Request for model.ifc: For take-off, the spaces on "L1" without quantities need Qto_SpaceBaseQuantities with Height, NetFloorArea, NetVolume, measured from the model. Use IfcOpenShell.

First a look at what the model holds.

```python
import ifcopenshell
import ifcopenshell.util.element
import ifcopenshell.util.unit

model = ifcopenshell.open("model.ifc")
print(model.schema)
for unit_type in ("LENGTHUNIT", "AREAUNIT", "VOLUMEUNIT"):
    print(unit_type, ifcopenshell.util.unit.calculate_unit_scale(model, unit_type))
storey = next(s for s in model.by_type("IfcBuildingStorey") if s.Name == "L1")
spaces = [e for e in ifcopenshell.util.element.get_decomposition(storey) if e.is_a("IfcSpace")]
for e in sorted(spaces, key=lambda e: e.id()):
    print(e.id(), e.is_a(), e.Name, list(ifcopenshell.util.element.get_psets(e, qtos_only=True)), sep=" | ")
```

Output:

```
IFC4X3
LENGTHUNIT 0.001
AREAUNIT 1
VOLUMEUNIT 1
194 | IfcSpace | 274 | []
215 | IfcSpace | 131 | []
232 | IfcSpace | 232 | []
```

```python
import ifcopenshell
import ifcopenshell.api.pset
import ifcopenshell.geom
import ifcopenshell.util.element
import ifcopenshell.util.shape
import ifcopenshell.util.unit

model = ifcopenshell.open("model.ifc")
unit_scale = ifcopenshell.util.unit.calculate_unit_scale(model)
area_scale = ifcopenshell.util.unit.calculate_unit_scale(model, "AREAUNIT")
volume_scale = ifcopenshell.util.unit.calculate_unit_scale(model, "VOLUMEUNIT")
settings = ifcopenshell.geom.settings()

storey = next(s for s in model.by_type("IfcBuildingStorey") if s.Name == "L1")
spaces = [e for e in ifcopenshell.util.element.get_decomposition(storey) if e.is_a("IfcSpace")]

for e in sorted(spaces, key=lambda e: e.id()):
    if ifcopenshell.util.element.get_psets(e, qtos_only=True, should_inherit=False):
        continue
    # Geometry comes back in metres, in the element's own axes.
    shape = ifcopenshell.geom.create_shape(settings, e)
    values = {
        "Height": ifcopenshell.util.shape.get_z(shape.geometry) / unit_scale,
        "NetFloorArea": ifcopenshell.util.shape.get_footprint_area(shape.geometry) / area_scale,
        "NetVolume": ifcopenshell.util.shape.get_volume(shape.geometry) / volume_scale,
    }
    qto = ifcopenshell.api.pset.add_qto(model, product=e, name="Qto_SpaceBaseQuantities")
    ifcopenshell.api.pset.edit_qto(model, qto=qto, properties=values)
    print(e.id(), {k: round(v, 3) for k, v in values.items()})

model.write("model_v2.ifc")
```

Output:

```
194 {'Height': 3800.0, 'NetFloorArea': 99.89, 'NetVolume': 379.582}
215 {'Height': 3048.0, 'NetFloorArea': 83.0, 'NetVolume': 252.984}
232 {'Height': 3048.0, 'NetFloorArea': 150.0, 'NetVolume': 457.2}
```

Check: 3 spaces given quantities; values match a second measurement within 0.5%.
